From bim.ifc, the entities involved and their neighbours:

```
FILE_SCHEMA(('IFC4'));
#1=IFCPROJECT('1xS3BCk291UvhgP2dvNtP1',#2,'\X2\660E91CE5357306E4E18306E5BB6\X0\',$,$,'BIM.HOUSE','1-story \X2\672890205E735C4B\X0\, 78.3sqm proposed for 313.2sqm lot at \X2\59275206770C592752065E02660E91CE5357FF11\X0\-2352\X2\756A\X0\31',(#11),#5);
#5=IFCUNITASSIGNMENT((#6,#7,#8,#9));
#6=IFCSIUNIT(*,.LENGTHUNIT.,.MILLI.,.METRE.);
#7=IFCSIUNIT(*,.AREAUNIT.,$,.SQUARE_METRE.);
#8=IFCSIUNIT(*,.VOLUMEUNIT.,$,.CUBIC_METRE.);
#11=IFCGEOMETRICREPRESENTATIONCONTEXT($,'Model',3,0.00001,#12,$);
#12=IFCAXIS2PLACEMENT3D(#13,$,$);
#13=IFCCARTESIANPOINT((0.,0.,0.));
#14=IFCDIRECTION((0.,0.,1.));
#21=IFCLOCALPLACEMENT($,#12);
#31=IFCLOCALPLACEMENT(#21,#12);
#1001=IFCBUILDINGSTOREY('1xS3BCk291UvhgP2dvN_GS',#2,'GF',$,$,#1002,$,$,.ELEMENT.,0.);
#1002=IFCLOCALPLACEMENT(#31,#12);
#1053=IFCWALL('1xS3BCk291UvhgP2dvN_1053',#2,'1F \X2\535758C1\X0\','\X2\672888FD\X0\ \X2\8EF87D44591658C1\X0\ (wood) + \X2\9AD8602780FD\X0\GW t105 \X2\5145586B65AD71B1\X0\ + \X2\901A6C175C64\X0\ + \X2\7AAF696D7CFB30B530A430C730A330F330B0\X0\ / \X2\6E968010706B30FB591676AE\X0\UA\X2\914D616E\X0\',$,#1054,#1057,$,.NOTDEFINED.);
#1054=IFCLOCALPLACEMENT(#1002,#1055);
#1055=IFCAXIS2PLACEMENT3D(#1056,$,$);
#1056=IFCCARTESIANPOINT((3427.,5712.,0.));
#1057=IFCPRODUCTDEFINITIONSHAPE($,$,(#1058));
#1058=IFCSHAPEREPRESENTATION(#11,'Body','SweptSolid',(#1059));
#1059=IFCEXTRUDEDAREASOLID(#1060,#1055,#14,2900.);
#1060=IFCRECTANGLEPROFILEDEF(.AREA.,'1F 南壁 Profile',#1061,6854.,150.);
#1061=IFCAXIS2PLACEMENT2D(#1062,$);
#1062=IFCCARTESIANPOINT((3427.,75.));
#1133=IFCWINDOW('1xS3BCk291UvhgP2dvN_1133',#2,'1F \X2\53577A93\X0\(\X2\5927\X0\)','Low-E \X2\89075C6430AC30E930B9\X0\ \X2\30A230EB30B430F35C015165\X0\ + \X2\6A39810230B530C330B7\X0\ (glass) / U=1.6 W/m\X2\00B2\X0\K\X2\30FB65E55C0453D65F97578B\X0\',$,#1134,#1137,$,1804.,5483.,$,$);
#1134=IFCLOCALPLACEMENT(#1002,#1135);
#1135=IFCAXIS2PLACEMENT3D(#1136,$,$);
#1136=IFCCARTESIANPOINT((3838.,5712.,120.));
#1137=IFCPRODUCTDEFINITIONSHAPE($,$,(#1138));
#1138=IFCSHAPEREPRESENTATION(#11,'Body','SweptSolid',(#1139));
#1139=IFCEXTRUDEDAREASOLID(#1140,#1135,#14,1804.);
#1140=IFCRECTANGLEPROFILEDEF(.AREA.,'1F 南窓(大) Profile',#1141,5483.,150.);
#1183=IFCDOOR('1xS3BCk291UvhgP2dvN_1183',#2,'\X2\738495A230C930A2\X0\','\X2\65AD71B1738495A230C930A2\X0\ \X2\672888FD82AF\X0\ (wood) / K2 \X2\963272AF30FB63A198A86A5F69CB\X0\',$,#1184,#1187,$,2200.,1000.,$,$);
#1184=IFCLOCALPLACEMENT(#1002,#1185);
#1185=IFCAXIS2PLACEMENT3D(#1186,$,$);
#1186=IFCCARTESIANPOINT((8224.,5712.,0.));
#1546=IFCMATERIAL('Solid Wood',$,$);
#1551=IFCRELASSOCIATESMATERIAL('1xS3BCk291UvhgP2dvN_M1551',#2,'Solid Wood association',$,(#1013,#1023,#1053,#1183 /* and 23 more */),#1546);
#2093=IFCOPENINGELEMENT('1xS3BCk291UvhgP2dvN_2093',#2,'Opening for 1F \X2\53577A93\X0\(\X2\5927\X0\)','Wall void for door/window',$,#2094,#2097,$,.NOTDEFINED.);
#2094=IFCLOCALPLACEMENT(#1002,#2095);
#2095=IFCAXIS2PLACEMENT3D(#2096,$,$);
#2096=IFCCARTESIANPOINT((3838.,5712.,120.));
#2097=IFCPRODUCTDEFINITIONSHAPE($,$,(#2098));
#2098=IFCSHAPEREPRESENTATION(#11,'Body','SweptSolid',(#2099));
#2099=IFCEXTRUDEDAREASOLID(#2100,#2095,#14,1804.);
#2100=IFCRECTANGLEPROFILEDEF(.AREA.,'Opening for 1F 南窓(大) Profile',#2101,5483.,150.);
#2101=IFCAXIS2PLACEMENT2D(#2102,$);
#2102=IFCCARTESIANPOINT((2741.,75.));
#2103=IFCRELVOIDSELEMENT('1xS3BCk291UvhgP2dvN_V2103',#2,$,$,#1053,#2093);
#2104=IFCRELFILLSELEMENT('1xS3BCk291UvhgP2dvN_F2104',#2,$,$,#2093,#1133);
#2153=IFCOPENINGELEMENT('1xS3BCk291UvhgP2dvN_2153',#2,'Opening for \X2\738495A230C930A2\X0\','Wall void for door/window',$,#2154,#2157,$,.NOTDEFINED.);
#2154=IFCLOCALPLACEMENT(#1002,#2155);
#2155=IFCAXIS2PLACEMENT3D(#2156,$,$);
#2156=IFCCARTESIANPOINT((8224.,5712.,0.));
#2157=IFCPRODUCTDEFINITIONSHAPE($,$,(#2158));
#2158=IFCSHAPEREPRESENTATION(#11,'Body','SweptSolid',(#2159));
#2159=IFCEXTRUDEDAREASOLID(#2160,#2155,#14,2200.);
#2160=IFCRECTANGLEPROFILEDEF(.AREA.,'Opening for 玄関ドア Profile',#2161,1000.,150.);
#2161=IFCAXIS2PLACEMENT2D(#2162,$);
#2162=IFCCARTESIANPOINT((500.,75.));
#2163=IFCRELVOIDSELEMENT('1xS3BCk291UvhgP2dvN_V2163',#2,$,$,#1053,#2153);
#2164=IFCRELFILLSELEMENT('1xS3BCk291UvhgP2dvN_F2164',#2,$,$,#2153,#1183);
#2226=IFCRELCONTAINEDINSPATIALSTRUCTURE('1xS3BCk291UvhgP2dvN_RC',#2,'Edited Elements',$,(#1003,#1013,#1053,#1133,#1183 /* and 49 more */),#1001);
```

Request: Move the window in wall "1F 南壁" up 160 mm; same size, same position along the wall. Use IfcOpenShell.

```python
import numpy as np
import ifcopenshell
import ifcopenshell.api.geometry
import ifcopenshell.util.placement
import ifcopenshell.util.unit

model = ifcopenshell.open("bim.ifc")
unit_scale = ifcopenshell.util.unit.calculate_unit_scale(model)

window = model.by_guid("1xS3BCk291UvhgP2dvN_1133")
opening = window.FillsVoids[0].RelatingOpeningElement
dz = 160.0

shift = np.array([0.0, 0.0, dz])
# The window is not placed relative to its opening, so move both.
for product in (opening, window):
    matrix = ifcopenshell.util.placement.get_local_placement(product.ObjectPlacement)
    matrix[:3, 3] += shift
    ifcopenshell.api.geometry.edit_object_placement(model, product=product, matrix=matrix, is_si=False)

print(f"moved by {dz * unit_scale:+.3f} m")

model.write("bim-out.ifc")
```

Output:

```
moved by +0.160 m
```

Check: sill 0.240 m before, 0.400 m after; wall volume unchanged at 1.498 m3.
